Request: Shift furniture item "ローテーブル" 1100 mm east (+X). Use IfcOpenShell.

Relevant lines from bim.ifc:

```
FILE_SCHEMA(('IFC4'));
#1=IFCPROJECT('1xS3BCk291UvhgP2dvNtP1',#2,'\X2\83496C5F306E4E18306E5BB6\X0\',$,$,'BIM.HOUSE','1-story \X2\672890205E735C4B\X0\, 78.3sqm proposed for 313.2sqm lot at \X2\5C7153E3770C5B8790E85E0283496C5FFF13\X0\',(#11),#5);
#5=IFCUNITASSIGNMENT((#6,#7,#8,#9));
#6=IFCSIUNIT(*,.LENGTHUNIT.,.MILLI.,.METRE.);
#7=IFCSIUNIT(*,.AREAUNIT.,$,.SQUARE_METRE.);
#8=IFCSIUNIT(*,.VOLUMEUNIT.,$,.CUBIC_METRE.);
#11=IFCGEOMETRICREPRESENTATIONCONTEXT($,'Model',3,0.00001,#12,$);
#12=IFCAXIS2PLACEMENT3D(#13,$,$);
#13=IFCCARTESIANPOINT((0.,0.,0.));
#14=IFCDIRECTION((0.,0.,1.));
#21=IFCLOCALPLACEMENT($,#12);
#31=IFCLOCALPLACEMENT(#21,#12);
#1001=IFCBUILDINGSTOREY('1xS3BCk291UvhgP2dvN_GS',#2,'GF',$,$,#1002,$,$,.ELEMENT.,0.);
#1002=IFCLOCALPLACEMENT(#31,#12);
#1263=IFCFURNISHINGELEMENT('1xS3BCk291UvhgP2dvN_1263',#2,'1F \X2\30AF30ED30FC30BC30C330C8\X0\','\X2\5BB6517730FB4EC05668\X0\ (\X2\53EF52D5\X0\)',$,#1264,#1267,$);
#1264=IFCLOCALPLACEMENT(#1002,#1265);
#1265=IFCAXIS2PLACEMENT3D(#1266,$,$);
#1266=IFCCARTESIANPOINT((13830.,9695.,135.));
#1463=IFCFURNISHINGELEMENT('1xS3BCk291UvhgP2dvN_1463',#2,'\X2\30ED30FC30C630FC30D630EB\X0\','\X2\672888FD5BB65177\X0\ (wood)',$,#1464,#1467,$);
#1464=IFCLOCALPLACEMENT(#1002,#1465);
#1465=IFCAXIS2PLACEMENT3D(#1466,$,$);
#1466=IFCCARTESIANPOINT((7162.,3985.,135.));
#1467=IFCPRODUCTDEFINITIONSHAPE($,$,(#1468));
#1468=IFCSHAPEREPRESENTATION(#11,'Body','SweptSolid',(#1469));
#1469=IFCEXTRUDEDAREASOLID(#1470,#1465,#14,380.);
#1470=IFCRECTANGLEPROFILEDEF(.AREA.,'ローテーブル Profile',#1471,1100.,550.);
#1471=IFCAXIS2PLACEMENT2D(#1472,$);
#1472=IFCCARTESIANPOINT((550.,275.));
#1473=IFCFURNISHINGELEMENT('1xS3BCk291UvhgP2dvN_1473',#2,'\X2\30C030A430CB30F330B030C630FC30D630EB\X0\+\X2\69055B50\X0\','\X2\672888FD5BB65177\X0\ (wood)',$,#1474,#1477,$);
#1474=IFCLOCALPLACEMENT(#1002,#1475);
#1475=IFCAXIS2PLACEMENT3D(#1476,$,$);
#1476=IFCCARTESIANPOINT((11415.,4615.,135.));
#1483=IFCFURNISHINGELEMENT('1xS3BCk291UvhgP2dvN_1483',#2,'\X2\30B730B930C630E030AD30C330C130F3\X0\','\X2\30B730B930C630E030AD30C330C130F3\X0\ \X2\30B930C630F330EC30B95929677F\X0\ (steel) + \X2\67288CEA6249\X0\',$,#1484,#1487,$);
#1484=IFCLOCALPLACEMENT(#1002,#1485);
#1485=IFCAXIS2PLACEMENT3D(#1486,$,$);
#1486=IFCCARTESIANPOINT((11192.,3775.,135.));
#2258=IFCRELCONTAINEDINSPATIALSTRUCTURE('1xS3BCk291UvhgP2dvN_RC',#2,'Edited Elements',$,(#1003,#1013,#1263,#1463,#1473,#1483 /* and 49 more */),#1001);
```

```python
import ifcopenshell
import ifcopenshell.api.geometry
import ifcopenshell.util.placement

model = ifcopenshell.open("bim.ifc")

item = model.by_id(1463)
matrix = ifcopenshell.util.placement.get_local_placement(item.ObjectPlacement)
matrix[0, 3] += 1100.0
ifcopenshell.api.geometry.edit_object_placement(model, product=item, matrix=matrix, is_si=False)

print(ifcopenshell.util.placement.get_local_placement(item.ObjectPlacement).round(3) + 0.0)

model.write("bim-out.ifc")
```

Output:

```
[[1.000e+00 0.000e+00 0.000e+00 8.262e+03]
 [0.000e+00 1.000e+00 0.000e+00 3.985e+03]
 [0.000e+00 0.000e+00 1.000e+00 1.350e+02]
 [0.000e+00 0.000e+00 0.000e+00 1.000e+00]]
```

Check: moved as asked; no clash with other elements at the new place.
